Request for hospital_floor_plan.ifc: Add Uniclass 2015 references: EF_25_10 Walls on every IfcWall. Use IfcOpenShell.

First a look at what the model holds.

```python
import ifcopenshell

model = ifcopenshell.open("hospital_floor_plan.ifc")
print(model.schema)
print("classifications:", [c.Name for c in model.by_type("IfcClassification")])
for ifc_class in ("IfcDoor", "IfcRoof", "IfcStair", "IfcWall", "IfcWindow"):
    print(ifc_class, len(model.by_type(ifc_class)))
```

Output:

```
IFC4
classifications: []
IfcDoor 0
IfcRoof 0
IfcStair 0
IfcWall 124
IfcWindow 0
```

```python
import ifcopenshell
import ifcopenshell.api.classification

model = ifcopenshell.open("hospital_floor_plan.ifc")

system = ifcopenshell.api.classification.add_classification(model, classification="Uniclass 2015")

codes = {
    "IfcWall": ("EF_25_10", "Walls"),
}
for ifc_class, (code, name) in codes.items():
    products = model.by_type(ifc_class)
    ifcopenshell.api.classification.add_reference(
        model, products=products, classification=system, identification=code, name=name
    )
    print(code, len(products))

model.write("hospital_floor_plan_edited.ifc")
```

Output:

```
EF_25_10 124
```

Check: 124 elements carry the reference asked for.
